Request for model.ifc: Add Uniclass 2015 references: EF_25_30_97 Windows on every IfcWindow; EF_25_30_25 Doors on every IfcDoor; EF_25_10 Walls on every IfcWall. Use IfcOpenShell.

First a look at what the model holds.

```python
import ifcopenshell

model = ifcopenshell.open("model.ifc")
print(model.schema)
print("classifications:", [c.Name for c in model.by_type("IfcClassification")])
for ifc_class in ("IfcDoor", "IfcRoof", "IfcStair", "IfcWall", "IfcWindow"):
    print(ifc_class, len(model.by_type(ifc_class)))
```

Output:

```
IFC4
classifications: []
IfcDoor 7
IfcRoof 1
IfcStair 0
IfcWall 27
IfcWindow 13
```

```python
import ifcopenshell
import ifcopenshell.api.classification

model = ifcopenshell.open("model.ifc")

system = ifcopenshell.api.classification.add_classification(model, classification="Uniclass 2015")

codes = {
    "IfcWindow": ("EF_25_30_97", "Windows"),
    "IfcDoor": ("EF_25_30_25", "Doors"),
    "IfcWall": ("EF_25_10", "Walls"),
}
for ifc_class, (code, name) in codes.items():
    products = model.by_type(ifc_class)
    ifcopenshell.api.classification.add_reference(
        model, products=products, classification=system, identification=code, name=name
    )
    print(code, len(products))

model.write("model_v2.ifc")
```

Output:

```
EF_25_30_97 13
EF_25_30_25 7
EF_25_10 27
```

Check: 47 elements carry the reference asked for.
